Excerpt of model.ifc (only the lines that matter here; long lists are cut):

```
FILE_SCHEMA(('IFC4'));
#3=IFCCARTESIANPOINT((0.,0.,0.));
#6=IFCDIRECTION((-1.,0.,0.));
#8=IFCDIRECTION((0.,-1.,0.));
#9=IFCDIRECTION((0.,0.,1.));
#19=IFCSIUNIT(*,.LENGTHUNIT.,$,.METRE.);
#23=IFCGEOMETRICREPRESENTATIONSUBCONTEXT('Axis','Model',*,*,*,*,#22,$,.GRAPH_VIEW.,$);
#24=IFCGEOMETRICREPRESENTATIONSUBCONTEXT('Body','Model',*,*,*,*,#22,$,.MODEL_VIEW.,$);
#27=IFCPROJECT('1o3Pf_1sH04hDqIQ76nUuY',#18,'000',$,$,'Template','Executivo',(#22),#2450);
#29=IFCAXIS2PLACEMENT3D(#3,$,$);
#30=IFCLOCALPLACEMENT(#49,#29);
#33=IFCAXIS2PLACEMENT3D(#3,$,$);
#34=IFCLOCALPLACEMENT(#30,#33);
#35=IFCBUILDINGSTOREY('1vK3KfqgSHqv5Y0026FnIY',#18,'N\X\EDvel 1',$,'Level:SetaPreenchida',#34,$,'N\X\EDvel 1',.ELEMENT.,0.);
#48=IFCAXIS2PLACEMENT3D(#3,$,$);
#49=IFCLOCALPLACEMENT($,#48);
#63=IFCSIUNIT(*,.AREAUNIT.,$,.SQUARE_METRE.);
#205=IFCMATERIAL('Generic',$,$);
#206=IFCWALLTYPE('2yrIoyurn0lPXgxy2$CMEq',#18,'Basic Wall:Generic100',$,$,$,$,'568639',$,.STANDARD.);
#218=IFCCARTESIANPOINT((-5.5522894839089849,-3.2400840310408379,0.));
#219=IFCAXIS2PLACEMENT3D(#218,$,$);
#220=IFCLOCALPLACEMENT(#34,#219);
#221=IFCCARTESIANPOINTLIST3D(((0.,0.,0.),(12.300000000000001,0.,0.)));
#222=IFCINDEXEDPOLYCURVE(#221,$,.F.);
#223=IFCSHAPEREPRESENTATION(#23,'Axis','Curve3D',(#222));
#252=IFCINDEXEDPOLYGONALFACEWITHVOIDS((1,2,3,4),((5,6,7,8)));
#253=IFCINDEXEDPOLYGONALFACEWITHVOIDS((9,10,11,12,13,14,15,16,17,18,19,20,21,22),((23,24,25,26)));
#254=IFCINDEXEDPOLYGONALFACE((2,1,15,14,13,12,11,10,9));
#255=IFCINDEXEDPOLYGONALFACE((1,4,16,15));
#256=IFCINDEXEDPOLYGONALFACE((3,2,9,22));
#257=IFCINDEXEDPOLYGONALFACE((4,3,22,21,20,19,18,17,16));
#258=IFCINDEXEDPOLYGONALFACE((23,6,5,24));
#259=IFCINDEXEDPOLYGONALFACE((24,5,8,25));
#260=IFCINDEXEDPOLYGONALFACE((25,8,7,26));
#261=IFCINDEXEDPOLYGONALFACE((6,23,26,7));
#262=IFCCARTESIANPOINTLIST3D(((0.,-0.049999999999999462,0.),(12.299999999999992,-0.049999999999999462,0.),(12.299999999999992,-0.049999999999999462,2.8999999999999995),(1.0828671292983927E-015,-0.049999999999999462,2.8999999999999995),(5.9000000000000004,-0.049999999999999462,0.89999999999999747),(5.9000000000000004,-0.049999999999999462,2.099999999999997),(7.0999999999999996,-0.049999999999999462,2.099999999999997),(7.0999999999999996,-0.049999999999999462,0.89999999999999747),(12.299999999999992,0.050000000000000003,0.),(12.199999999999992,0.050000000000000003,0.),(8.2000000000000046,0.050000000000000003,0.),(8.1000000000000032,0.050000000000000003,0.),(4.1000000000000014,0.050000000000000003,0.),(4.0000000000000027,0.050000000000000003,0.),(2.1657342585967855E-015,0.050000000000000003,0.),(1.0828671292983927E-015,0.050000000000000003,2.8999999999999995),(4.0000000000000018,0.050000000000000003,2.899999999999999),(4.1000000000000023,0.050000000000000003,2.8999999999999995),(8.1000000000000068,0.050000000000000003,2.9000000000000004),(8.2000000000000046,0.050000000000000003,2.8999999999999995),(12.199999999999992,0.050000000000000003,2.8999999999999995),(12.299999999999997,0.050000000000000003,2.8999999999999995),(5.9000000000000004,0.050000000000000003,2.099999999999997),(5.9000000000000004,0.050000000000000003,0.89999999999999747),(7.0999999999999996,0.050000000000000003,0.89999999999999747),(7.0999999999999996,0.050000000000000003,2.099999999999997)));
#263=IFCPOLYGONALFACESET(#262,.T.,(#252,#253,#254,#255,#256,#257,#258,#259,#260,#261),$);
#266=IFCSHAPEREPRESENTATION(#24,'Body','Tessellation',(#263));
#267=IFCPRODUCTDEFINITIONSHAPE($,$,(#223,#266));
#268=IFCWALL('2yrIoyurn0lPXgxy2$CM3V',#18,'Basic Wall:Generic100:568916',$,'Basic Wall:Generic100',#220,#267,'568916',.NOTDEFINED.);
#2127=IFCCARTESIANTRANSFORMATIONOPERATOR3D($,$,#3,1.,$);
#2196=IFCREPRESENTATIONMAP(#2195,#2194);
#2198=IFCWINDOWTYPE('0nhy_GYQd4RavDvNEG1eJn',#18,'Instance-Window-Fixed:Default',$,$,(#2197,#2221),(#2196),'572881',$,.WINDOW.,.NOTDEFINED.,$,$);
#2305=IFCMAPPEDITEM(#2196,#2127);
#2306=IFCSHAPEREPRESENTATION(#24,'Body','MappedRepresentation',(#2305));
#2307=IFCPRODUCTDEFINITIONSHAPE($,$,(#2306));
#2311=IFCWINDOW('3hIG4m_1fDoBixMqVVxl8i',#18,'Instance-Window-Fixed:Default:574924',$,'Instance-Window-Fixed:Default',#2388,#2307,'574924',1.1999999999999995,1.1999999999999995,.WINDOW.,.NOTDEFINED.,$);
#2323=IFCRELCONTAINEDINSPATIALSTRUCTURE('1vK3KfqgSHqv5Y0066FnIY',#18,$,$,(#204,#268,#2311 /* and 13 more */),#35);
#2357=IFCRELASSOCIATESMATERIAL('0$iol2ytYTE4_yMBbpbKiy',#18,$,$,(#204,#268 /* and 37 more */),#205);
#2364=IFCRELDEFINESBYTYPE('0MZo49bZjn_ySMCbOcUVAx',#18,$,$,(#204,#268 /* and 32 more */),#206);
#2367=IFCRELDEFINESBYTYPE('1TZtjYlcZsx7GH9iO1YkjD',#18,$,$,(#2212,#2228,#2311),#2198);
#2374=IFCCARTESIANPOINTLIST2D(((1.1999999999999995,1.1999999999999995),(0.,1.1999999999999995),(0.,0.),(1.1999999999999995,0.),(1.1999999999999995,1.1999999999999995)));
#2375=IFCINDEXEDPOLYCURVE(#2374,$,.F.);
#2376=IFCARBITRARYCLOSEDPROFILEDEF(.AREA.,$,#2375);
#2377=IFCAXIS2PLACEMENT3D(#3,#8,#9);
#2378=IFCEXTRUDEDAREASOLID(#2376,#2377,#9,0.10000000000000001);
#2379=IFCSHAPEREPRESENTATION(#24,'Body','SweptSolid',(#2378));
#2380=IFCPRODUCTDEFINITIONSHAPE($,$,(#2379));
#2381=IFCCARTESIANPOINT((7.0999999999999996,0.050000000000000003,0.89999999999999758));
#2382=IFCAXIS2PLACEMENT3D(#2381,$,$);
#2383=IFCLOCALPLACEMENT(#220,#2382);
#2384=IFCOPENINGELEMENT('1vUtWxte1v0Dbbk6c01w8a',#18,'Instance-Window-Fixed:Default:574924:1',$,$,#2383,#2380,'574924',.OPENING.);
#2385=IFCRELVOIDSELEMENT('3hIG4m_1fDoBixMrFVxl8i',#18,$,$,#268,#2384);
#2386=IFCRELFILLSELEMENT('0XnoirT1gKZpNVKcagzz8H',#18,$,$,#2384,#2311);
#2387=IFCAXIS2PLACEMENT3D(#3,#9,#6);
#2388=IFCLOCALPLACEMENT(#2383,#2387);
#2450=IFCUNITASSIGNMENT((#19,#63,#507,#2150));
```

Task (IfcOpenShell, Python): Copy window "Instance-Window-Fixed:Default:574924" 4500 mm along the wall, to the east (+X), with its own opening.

```python
import ifcopenshell
import ifcopenshell.api.feature
import ifcopenshell.api.geometry
import ifcopenshell.api.root
import ifcopenshell.geom
import ifcopenshell.util.element
import ifcopenshell.util.placement
import ifcopenshell.util.shape
import ifcopenshell.util.unit

model = ifcopenshell.open("model.ifc")
unit_scale = ifcopenshell.util.unit.calculate_unit_scale(model)
settings = ifcopenshell.geom.settings()


def volume(element):
    """Net volume in cubic metres, openings subtracted."""
    shape = ifcopenshell.geom.create_shape(settings, element)
    return ifcopenshell.util.shape.get_volume(shape.geometry)


def reuse_history(source, copy):
    """copy_class also copies each property set's owner history, people and application; keep the originals."""
    for rel in copy.IsDefinedBy:
        if rel.is_a("IfcRelDefinesByProperties") and (history := rel.RelatingPropertyDefinition.OwnerHistory):
            rel.RelatingPropertyDefinition.OwnerHistory = source.OwnerHistory
            ifcopenshell.util.element.remove_deep2(model, history)


window = model.by_guid("3hIG4m_1fDoBixMqVVxl8i")
opening = window.FillsVoids[0].RelatingOpeningElement
wall = opening.VoidsElements[0].RelatingBuildingElement
before = volume(wall)
shift = ifcopenshell.util.placement.get_local_placement(wall.ObjectPlacement)[:3, 0] * 4.5 / unit_scale

# copy_class copies the void relationship, type, container and properties, but no geometry.
new_opening = ifcopenshell.api.root.copy_class(model, product=opening)
new_opening.Representation = ifcopenshell.util.element.copy_deep(
    model, opening.Representation, exclude=["IfcGeometricRepresentationContext", "IfcRepresentationMap"]
)
new_opening.Name = "Instance-Window-Fixed:Default"
new_opening.Tag = None
new_window = ifcopenshell.api.root.copy_class(model, product=window)
new_window.Representation = ifcopenshell.util.element.copy_deep(
    model, window.Representation, exclude=["IfcGeometricRepresentationContext", "IfcRepresentationMap"]
)
new_window.Name = "Instance-Window-Fixed:Default"
new_window.Tag = None
reuse_history(window, new_window)
ifcopenshell.api.feature.add_filling(model, opening=new_opening, element=new_window)

for old, new in ((opening, new_opening), (window, new_window)):
    matrix = ifcopenshell.util.placement.get_local_placement(old.ObjectPlacement)
    matrix[:3, 3] += shift
    ifcopenshell.api.geometry.edit_object_placement(model, product=new, matrix=matrix, is_si=False)

after = volume(wall)

print(f"wall volume {before:.3f} -> {after:.3f} m3")

model.write("model_edited.ifc")
```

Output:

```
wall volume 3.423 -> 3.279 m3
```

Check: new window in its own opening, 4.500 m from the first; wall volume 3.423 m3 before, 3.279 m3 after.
